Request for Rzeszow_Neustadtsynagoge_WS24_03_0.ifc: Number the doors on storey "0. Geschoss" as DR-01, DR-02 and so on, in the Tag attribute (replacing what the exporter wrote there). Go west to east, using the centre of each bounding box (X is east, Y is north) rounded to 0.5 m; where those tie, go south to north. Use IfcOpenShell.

First a look at what the model holds.

```python
import ifcopenshell
import ifcopenshell.util.element
import ifcopenshell.util.placement

model = ifcopenshell.open("Rzeszow_Neustadtsynagoge_WS24_03_0.ifc")
print(model.schema)
storey = next(s for s in model.by_type("IfcBuildingStorey") if s.Name == "0. Geschoss")
doors = [e for e in ifcopenshell.util.element.get_decomposition(storey) if e.is_a("IfcDoor")]
for e in sorted(doors, key=lambda e: e.id()):
    origin = ifcopenshell.util.placement.get_local_placement(e.ObjectPlacement)[:3, 3]
    print(e.id(), e.Tag, e.Name, origin.round(2) + 0.0, sep=" | ")
```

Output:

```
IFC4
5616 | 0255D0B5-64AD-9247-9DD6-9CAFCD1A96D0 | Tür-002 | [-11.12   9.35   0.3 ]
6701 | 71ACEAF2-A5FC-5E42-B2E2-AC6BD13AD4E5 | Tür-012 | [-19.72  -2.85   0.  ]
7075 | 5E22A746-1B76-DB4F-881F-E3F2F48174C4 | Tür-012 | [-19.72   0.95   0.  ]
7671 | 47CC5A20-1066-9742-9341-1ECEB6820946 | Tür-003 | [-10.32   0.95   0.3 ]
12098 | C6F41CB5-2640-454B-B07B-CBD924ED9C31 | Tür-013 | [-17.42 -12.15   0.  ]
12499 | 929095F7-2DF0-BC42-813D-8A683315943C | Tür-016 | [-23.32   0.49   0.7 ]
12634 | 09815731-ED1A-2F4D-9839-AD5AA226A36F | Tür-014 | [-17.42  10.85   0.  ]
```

```python
import ifcopenshell
import ifcopenshell.geom
import ifcopenshell.util.element
import ifcopenshell.util.shape

model = ifcopenshell.open("Rzeszow_Neustadtsynagoge_WS24_03_0.ifc")
settings = ifcopenshell.geom.settings()
settings.set("use-world-coords", True)


def centre(element):
    shape = ifcopenshell.geom.create_shape(settings, element)
    return ifcopenshell.util.shape.get_bbox_centroid(shape.geometry)


storey = next(s for s in model.by_type("IfcBuildingStorey") if s.Name == "0. Geschoss")
doors = [e for e in ifcopenshell.util.element.get_decomposition(storey) if e.is_a("IfcDoor")]

# Insertion points can sit at a corner or the storey origin, so sort by the geometry (in metres).
centres = {e: centre(e) for e in doors}
doors.sort(key=lambda e: (round(centres[e][0] / 0.5), centres[e][1]))

for i, e in enumerate(doors, start=1):
    number = f"DR-{i:02d}"
    e.Tag = number
    print(e.id(), number)

model.write("Rzeszow_Neustadtsynagoge_WS24_03_0-out.ifc")
```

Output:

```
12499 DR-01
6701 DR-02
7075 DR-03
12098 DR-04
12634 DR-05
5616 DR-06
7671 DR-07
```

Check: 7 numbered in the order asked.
